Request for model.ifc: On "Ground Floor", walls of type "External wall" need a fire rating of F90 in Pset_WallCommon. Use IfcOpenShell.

First a look at what the model holds.

```python
import ifcopenshell
import ifcopenshell.util.element

model = ifcopenshell.open("model.ifc")
print(model.schema)
storey = next(s for s in model.by_type("IfcBuildingStorey") if s.Name == "Ground Floor")
walls = [e for e in ifcopenshell.util.element.get_decomposition(storey) if e.is_a("IfcWall")]
seen = {}
for e in walls:
    element_type = ifcopenshell.util.element.get_type(e)
    key = (element_type.Name if element_type != e and element_type else None, ifcopenshell.util.element.get_pset(e, "Pset_WallCommon", "FireRating"))
    seen[key] = seen.get(key, 0) + 1
for (name, value), count in sorted(seen.items(), key=str):
    print(count, "x", name, "|", value)
```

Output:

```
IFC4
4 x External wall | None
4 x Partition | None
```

```python
import ifcopenshell
import ifcopenshell.api.pset
import ifcopenshell.util.element

model = ifcopenshell.open("model.ifc")

storey = next(s for s in model.by_type("IfcBuildingStorey") if s.Name == "Ground Floor")
walls = [e for e in ifcopenshell.util.element.get_decomposition(storey) if e.is_a("IfcWall")]

count = 0
for e in walls:
    element_type = ifcopenshell.util.element.get_type(e)
    if element_type in (None, e) or element_type.Name != "External wall":
        continue
    # add_pset returns the element's existing set when there is one.
    pset = ifcopenshell.api.pset.add_pset(model, product=e, name="Pset_WallCommon")
    ifcopenshell.api.pset.edit_pset(model, pset=pset, properties={"FireRating": "F90"})
    count += 1

print(count, "walls updated")

model.write("model_edited.ifc")
```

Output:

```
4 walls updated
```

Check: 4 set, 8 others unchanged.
